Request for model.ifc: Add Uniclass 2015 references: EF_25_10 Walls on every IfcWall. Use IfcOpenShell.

First a look at what the model holds.

```python
import ifcopenshell

model = ifcopenshell.open("model.ifc")
print(model.schema)
print("classifications:", [c.Name for c in model.by_type("IfcClassification")])
for ifc_class in ("IfcDoor", "IfcRoof", "IfcStair", "IfcWall", "IfcWindow"):
    print(ifc_class, len(model.by_type(ifc_class)))
```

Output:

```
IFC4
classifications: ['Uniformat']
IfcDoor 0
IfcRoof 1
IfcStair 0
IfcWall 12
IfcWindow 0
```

```python
import ifcopenshell
import ifcopenshell.api.classification

model = ifcopenshell.open("model.ifc")

system = ifcopenshell.api.classification.add_classification(model, classification="Uniclass 2015")

codes = {
    "IfcWall": ("EF_25_10", "Walls"),
}
for ifc_class, (code, name) in codes.items():
    products = model.by_type(ifc_class)
    ifcopenshell.api.classification.add_reference(
        model, products=products, classification=system, identification=code, name=name
    )
    print(code, len(products))

model.write("model_edited.ifc")
```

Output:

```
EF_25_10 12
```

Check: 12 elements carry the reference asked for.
